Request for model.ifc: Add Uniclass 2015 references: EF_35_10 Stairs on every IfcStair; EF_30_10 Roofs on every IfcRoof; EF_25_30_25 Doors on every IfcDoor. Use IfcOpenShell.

First a look at what the model holds.

```python
import ifcopenshell

model = ifcopenshell.open("model.ifc")
print(model.schema)
print("classifications:", [c.Name for c in model.by_type("IfcClassification")])
for ifc_class in ("IfcDoor", "IfcRoof", "IfcStair", "IfcWall", "IfcWindow"):
    print(ifc_class, len(model.by_type(ifc_class)))
```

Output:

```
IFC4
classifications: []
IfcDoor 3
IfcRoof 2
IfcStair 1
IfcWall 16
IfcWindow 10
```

```python
import ifcopenshell
import ifcopenshell.api.classification

model = ifcopenshell.open("model.ifc")

system = ifcopenshell.api.classification.add_classification(model, classification="Uniclass 2015")

codes = {
    "IfcStair": ("EF_35_10", "Stairs"),
    "IfcRoof": ("EF_30_10", "Roofs"),
    "IfcDoor": ("EF_25_30_25", "Doors"),
}
for ifc_class, (code, name) in codes.items():
    products = model.by_type(ifc_class)
    ifcopenshell.api.classification.add_reference(
        model, products=products, classification=system, identification=code, name=name
    )
    print(code, len(products))

model.write("model_edited.ifc")
```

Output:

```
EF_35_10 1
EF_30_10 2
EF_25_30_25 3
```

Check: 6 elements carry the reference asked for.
